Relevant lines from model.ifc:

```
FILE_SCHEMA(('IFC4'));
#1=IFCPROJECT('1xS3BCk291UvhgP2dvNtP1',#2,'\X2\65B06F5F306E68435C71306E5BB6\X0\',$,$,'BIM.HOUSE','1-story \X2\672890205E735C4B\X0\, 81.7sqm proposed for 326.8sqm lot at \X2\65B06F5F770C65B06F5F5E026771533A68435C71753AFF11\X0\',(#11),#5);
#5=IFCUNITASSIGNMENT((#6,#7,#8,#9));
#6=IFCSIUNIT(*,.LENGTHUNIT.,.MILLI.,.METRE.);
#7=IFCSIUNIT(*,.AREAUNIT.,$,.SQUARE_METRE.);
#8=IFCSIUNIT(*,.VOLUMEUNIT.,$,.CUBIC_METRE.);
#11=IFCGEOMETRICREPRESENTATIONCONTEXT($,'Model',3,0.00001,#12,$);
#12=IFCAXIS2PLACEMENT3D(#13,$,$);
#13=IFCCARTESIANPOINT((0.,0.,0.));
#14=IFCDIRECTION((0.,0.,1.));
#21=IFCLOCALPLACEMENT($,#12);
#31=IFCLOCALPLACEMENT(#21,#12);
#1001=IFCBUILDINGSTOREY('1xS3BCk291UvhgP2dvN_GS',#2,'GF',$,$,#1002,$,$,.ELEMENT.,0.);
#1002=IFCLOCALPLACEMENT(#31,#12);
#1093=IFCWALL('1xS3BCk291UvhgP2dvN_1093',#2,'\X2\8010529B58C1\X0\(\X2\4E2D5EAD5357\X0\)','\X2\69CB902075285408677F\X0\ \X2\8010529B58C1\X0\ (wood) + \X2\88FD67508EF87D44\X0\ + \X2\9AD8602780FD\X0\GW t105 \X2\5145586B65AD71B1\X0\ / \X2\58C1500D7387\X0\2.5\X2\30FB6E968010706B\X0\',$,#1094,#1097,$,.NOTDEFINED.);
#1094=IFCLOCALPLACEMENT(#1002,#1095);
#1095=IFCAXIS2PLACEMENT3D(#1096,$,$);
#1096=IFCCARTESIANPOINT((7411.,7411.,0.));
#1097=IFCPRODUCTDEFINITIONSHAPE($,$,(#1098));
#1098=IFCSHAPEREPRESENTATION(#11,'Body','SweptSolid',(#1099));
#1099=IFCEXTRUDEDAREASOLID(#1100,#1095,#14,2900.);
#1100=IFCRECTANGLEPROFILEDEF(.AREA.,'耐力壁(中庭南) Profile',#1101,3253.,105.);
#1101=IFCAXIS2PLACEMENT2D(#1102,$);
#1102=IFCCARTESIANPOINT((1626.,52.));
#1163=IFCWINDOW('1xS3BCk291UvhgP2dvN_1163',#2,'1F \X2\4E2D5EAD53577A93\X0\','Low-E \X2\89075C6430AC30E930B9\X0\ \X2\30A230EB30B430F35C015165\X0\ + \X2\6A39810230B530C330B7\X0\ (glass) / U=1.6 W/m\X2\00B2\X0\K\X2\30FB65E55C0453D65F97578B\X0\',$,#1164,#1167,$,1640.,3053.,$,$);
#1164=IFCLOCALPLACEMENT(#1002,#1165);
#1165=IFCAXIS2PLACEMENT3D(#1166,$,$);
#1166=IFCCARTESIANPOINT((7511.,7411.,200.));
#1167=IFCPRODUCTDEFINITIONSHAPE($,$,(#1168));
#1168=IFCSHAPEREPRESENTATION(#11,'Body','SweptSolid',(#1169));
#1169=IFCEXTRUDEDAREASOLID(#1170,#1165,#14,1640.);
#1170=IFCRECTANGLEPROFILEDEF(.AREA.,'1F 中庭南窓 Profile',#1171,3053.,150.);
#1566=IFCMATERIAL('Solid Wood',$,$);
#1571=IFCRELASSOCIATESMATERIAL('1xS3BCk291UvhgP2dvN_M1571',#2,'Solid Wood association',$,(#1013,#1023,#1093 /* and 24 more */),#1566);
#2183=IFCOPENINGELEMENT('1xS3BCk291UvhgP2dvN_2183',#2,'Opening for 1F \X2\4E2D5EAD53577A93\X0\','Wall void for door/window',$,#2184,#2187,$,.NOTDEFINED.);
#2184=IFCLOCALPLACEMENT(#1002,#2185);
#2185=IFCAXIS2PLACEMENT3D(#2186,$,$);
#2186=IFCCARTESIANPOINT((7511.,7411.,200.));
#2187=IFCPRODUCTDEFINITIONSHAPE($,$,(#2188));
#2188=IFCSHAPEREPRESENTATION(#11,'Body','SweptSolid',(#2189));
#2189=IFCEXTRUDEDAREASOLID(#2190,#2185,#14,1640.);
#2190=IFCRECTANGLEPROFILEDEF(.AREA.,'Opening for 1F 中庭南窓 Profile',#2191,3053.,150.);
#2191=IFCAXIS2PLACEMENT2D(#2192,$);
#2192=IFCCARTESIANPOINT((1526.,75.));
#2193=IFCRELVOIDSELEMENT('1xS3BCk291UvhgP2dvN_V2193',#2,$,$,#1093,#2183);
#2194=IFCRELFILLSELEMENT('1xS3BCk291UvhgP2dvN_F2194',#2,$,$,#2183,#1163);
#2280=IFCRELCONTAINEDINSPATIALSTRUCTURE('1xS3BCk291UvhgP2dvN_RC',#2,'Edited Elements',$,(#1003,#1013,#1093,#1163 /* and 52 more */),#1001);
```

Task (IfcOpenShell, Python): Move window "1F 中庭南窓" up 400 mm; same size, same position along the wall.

```python
import numpy as np
import ifcopenshell
import ifcopenshell.api.geometry
import ifcopenshell.util.placement
import ifcopenshell.util.unit

model = ifcopenshell.open("model.ifc")
unit_scale = ifcopenshell.util.unit.calculate_unit_scale(model)

window = model.by_guid("1xS3BCk291UvhgP2dvN_1163")
opening = window.FillsVoids[0].RelatingOpeningElement
dz = 400.0

shift = np.array([0.0, 0.0, dz])
# The window is not placed relative to its opening, so move both.
for product in (opening, window):
    matrix = ifcopenshell.util.placement.get_local_placement(product.ObjectPlacement)
    matrix[:3, 3] += shift
    ifcopenshell.api.geometry.edit_object_placement(model, product=product, matrix=matrix, is_si=False)

print(f"moved by {dz * unit_scale:+.3f} m")

model.write("model_rev.ifc")
```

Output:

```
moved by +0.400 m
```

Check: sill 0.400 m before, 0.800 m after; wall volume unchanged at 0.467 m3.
